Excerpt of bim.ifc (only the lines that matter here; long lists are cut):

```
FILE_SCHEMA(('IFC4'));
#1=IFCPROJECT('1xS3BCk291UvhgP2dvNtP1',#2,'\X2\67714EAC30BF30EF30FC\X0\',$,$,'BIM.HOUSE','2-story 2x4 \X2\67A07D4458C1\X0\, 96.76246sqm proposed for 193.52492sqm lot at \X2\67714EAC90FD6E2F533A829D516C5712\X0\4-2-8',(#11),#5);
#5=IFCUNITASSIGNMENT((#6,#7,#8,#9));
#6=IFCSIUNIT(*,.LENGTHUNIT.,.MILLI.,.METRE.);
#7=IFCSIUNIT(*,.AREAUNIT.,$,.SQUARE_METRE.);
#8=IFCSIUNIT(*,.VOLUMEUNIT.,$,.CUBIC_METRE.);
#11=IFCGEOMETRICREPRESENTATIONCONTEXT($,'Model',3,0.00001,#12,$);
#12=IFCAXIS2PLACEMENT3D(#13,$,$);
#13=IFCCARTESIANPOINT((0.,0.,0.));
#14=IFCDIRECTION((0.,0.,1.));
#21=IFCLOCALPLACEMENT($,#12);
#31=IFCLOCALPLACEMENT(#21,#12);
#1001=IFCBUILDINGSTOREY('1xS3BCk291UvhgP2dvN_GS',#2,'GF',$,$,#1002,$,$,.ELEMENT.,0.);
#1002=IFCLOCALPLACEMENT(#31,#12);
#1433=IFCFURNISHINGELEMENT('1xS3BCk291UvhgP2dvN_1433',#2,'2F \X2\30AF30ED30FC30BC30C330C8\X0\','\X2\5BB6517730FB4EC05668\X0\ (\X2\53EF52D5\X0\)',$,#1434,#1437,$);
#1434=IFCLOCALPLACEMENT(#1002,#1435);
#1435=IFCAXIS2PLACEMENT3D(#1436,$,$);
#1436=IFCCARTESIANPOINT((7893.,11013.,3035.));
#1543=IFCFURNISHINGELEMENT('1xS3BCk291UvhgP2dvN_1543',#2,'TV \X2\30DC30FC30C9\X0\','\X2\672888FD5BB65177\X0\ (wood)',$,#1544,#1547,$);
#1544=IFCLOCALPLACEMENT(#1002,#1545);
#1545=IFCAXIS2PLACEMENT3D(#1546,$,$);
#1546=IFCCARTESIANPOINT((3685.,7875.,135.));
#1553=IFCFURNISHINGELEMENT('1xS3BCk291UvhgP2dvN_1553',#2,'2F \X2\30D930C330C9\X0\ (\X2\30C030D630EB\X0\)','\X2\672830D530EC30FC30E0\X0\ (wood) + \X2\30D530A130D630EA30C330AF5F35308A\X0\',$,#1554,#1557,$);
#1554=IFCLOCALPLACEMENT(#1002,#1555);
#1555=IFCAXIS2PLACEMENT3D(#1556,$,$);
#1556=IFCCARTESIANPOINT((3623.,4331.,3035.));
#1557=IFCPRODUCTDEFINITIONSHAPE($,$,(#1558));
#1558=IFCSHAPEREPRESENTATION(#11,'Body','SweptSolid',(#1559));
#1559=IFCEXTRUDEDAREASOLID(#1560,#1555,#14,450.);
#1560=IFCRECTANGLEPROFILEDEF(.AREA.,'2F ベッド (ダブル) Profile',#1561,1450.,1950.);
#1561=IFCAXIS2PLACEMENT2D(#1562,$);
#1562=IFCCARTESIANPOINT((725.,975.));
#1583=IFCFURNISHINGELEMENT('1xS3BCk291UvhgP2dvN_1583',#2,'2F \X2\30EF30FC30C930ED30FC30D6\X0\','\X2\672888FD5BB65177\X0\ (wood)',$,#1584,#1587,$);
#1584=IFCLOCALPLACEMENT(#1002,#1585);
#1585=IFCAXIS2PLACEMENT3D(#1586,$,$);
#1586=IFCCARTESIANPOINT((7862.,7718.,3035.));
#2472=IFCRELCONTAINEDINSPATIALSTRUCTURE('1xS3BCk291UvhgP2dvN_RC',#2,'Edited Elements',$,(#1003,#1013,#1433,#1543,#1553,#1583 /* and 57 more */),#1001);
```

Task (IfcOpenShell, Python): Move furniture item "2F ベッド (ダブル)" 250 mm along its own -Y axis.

```python
import ifcopenshell
import ifcopenshell.api.geometry
import ifcopenshell.util.placement
import ifcopenshell.util.unit

model = ifcopenshell.open("bim.ifc")
unit_scale = ifcopenshell.util.unit.calculate_unit_scale(model)

item = model.by_guid("1xS3BCk291UvhgP2dvN_1553")
matrix = ifcopenshell.util.placement.get_local_placement(item.ObjectPlacement)
matrix[:3, 3] -= matrix[:3, 1] * 0.25 / unit_scale
ifcopenshell.api.geometry.edit_object_placement(model, product=item, matrix=matrix, is_si=False)

print(ifcopenshell.util.placement.get_local_placement(item.ObjectPlacement).round(3) + 0.0)

model.write("bim_v2.ifc")
```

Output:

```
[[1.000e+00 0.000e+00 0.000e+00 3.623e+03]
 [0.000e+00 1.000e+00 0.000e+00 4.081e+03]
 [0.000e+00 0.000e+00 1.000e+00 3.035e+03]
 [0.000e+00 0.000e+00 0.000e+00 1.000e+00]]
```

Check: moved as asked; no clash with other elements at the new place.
